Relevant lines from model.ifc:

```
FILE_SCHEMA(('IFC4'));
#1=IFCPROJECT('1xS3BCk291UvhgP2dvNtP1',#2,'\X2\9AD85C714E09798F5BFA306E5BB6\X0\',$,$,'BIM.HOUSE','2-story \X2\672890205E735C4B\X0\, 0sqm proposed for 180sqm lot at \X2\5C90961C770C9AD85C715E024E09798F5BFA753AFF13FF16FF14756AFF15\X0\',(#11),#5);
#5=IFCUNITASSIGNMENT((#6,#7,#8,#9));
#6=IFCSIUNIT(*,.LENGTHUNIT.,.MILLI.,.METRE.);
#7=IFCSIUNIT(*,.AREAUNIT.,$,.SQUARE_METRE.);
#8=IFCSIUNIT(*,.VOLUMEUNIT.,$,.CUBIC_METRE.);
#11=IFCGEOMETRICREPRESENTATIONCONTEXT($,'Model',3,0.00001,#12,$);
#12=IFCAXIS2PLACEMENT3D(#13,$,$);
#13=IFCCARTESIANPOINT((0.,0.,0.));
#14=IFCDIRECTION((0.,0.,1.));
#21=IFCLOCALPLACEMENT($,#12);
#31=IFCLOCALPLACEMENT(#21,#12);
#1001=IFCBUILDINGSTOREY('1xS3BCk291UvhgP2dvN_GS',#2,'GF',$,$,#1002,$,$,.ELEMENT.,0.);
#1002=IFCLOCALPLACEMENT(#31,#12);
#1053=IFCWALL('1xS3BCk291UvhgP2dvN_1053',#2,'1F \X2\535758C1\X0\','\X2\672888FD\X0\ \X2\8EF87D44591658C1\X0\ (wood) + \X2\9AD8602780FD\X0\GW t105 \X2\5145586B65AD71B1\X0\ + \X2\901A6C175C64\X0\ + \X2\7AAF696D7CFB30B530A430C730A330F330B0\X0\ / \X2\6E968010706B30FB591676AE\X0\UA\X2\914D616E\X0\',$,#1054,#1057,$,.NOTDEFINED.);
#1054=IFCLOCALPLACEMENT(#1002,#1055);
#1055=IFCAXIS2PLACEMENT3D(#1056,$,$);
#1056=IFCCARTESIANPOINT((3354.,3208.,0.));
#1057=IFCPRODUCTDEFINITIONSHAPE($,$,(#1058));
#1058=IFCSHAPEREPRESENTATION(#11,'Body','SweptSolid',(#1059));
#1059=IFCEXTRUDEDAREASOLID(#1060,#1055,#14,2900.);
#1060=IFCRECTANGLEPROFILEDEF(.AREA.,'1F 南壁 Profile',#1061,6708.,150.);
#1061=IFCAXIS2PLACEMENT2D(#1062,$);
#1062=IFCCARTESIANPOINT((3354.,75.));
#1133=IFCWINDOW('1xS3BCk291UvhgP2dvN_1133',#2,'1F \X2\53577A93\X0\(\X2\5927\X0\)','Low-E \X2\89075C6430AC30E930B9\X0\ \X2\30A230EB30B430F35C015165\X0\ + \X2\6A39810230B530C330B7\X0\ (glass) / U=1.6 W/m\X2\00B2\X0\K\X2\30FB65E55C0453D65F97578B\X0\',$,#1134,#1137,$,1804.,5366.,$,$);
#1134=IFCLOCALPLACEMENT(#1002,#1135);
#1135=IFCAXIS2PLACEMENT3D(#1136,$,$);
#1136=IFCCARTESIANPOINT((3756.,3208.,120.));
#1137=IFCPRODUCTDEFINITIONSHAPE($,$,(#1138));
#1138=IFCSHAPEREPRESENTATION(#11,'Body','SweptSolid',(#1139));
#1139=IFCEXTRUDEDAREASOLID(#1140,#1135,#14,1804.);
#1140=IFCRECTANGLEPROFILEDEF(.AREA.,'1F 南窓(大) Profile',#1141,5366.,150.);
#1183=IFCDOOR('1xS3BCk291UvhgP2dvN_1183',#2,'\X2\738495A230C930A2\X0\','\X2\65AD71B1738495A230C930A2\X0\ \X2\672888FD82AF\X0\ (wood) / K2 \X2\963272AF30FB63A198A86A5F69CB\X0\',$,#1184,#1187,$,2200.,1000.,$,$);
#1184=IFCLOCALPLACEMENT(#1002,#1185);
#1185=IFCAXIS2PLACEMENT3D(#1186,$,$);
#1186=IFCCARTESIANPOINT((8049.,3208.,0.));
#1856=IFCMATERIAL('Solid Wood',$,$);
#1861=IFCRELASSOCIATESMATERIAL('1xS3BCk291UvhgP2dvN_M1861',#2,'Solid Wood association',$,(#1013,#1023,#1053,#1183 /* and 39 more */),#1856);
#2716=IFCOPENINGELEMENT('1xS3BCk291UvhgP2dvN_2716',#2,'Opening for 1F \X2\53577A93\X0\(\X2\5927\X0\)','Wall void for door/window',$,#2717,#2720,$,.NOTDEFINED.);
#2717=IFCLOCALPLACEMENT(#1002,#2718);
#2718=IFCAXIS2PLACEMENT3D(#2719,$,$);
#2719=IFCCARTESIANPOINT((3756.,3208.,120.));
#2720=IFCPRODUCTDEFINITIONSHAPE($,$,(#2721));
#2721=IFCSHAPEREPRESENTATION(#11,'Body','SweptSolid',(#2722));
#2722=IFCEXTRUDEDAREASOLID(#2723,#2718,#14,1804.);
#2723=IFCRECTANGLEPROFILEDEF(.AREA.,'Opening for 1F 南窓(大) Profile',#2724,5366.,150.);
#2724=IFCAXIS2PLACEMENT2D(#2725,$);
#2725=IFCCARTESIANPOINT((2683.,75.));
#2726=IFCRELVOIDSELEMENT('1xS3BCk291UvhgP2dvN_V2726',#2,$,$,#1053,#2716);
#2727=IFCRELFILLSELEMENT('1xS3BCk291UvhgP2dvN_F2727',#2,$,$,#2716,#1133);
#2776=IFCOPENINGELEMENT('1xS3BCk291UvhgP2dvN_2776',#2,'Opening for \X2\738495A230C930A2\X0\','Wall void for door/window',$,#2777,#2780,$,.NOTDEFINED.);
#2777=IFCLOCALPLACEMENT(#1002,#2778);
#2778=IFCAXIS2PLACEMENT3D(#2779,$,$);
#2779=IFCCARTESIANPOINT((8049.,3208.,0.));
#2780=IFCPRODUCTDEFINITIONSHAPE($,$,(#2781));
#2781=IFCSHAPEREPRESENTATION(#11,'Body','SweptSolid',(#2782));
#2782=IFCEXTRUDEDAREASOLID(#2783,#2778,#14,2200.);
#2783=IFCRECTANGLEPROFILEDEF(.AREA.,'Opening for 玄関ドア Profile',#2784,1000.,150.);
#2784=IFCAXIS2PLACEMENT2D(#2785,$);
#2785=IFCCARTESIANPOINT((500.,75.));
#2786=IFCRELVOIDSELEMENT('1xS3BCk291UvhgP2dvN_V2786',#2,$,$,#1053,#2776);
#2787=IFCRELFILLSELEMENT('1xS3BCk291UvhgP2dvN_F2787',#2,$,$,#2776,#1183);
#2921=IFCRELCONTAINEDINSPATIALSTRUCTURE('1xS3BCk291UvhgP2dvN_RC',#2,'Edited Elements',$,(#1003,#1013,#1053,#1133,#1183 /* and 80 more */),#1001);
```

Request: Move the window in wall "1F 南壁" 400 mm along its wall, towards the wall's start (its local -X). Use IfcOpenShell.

```python
import ifcopenshell
import ifcopenshell.api.geometry
import ifcopenshell.util.placement

model = ifcopenshell.open("model.ifc")

window = model.by_guid("1xS3BCk291UvhgP2dvN_1133")
opening = window.FillsVoids[0].RelatingOpeningElement
wall = opening.VoidsElements[0].RelatingBuildingElement

wall_matrix = ifcopenshell.util.placement.get_local_placement(wall.ObjectPlacement)
shift = wall_matrix[:3, 0] * -400.0
before = ifcopenshell.util.placement.get_local_placement(window.ObjectPlacement)[:3, 3].copy()

# The window is not placed relative to its opening, so move both.
for product in (opening, window):
    matrix = ifcopenshell.util.placement.get_local_placement(product.ObjectPlacement)
    matrix[:3, 3] += shift
    ifcopenshell.api.geometry.edit_object_placement(model, product=product, matrix=matrix, is_si=False)

after = ifcopenshell.util.placement.get_local_placement(window.ObjectPlacement)[:3, 3]
print("window moved by", (after - before).round(3) + 0.0)

model.write("model_edited.ifc")
```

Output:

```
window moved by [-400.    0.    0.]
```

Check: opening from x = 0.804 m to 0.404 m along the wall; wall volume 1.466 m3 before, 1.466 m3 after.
